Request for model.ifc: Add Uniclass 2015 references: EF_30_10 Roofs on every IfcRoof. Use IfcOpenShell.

First a look at what the model holds.

```python
import ifcopenshell

model = ifcopenshell.open("model.ifc")
print(model.schema)
print("classifications:", [c.Name for c in model.by_type("IfcClassification")])
for ifc_class in ("IfcDoor", "IfcRoof", "IfcStair", "IfcWall", "IfcWindow"):
    print(ifc_class, len(model.by_type(ifc_class)))
```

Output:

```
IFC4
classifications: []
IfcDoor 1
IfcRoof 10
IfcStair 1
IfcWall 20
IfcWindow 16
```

```python
import ifcopenshell
import ifcopenshell.api.classification

model = ifcopenshell.open("model.ifc")

system = ifcopenshell.api.classification.add_classification(model, classification="Uniclass 2015")

codes = {
    "IfcRoof": ("EF_30_10", "Roofs"),
}
for ifc_class, (code, name) in codes.items():
    products = model.by_type(ifc_class)
    ifcopenshell.api.classification.add_reference(
        model, products=products, classification=system, identification=code, name=name
    )
    print(code, len(products))

model.write("model_updated.ifc")
```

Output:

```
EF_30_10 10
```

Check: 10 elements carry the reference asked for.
